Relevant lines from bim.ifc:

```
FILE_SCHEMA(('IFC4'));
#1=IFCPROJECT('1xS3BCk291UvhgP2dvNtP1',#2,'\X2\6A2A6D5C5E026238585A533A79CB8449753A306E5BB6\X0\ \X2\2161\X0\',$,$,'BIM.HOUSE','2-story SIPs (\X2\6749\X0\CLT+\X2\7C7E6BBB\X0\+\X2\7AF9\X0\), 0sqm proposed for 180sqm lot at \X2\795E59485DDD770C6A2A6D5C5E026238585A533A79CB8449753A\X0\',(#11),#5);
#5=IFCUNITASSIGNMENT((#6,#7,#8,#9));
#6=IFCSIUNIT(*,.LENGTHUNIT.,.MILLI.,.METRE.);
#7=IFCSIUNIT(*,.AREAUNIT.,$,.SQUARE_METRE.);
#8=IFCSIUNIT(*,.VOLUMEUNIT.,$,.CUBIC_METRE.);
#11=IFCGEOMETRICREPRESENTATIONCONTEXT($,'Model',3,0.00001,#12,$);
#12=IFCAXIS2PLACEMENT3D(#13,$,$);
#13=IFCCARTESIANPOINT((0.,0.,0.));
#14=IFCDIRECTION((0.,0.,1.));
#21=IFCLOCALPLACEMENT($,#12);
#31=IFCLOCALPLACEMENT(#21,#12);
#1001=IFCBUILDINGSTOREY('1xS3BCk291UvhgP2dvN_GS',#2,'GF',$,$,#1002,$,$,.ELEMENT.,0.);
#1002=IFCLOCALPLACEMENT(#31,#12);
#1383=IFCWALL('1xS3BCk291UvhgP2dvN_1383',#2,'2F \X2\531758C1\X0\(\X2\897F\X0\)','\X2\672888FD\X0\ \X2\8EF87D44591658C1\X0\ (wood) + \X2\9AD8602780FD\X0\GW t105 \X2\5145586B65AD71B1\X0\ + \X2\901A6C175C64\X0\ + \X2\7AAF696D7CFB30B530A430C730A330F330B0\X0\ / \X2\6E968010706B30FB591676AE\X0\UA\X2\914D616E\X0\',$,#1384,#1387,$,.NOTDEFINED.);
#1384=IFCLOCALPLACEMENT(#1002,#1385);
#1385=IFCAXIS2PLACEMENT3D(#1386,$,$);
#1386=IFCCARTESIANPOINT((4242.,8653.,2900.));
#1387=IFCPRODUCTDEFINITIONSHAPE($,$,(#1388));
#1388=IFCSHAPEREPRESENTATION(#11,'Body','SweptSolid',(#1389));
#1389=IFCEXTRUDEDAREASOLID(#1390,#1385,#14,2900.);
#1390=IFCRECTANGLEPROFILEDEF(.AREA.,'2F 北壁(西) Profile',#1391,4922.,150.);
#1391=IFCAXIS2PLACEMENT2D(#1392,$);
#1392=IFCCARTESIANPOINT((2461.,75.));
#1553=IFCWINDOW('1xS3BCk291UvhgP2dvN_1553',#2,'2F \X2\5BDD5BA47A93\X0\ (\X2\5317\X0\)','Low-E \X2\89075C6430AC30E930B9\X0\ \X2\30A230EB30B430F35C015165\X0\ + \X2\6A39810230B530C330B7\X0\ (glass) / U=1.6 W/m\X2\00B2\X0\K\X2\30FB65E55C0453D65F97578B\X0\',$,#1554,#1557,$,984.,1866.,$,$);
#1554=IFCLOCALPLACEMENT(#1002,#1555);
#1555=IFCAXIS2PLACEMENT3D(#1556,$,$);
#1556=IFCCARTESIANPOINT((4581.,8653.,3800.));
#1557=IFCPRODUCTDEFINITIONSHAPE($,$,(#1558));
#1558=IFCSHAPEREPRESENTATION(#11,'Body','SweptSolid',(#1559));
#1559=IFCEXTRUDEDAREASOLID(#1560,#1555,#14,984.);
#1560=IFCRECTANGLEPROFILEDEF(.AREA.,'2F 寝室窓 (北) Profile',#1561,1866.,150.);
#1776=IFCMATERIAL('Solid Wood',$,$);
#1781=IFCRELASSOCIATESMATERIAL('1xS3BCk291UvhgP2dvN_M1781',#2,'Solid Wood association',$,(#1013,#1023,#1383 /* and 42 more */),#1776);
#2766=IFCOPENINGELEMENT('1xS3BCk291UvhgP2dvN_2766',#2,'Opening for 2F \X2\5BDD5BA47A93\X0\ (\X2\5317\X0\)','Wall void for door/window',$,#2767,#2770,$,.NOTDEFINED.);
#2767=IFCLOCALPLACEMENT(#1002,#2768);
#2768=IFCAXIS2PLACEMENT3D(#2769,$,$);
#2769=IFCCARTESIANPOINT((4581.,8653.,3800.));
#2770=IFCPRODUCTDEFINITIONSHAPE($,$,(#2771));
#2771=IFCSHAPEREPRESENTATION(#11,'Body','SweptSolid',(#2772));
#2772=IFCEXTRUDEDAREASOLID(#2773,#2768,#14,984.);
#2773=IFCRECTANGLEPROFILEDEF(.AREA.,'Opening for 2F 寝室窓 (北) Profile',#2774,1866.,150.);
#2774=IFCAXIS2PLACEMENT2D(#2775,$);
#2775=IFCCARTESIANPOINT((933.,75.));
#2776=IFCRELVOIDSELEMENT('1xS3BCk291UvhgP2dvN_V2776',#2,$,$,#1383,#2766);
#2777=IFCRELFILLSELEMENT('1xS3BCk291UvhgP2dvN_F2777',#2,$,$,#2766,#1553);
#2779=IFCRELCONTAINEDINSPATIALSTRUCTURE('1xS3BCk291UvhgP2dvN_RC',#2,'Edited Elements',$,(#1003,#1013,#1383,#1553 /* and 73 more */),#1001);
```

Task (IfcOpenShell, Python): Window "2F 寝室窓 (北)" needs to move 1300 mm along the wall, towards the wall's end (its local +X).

```python
import ifcopenshell
import ifcopenshell.api.geometry
import ifcopenshell.util.placement
import ifcopenshell.util.unit

model = ifcopenshell.open("bim.ifc")
unit_scale = ifcopenshell.util.unit.calculate_unit_scale(model)

window = model.by_guid("1xS3BCk291UvhgP2dvN_1553")
opening = window.FillsVoids[0].RelatingOpeningElement
wall = opening.VoidsElements[0].RelatingBuildingElement

wall_matrix = ifcopenshell.util.placement.get_local_placement(wall.ObjectPlacement)
shift = wall_matrix[:3, 0] * 1.3 / unit_scale
before = ifcopenshell.util.placement.get_local_placement(window.ObjectPlacement)[:3, 3].copy()

# The window is not placed relative to its opening, so move both.
for product in (opening, window):
    matrix = ifcopenshell.util.placement.get_local_placement(product.ObjectPlacement)
    matrix[:3, 3] += shift
    ifcopenshell.api.geometry.edit_object_placement(model, product=product, matrix=matrix, is_si=False)

after = ifcopenshell.util.placement.get_local_placement(window.ObjectPlacement)[:3, 3]
print("window moved by", (after - before).round(3) + 0.0)

model.write("bim_edited.ifc")
```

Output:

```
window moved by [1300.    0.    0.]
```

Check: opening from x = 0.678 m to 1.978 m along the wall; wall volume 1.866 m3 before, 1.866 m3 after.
